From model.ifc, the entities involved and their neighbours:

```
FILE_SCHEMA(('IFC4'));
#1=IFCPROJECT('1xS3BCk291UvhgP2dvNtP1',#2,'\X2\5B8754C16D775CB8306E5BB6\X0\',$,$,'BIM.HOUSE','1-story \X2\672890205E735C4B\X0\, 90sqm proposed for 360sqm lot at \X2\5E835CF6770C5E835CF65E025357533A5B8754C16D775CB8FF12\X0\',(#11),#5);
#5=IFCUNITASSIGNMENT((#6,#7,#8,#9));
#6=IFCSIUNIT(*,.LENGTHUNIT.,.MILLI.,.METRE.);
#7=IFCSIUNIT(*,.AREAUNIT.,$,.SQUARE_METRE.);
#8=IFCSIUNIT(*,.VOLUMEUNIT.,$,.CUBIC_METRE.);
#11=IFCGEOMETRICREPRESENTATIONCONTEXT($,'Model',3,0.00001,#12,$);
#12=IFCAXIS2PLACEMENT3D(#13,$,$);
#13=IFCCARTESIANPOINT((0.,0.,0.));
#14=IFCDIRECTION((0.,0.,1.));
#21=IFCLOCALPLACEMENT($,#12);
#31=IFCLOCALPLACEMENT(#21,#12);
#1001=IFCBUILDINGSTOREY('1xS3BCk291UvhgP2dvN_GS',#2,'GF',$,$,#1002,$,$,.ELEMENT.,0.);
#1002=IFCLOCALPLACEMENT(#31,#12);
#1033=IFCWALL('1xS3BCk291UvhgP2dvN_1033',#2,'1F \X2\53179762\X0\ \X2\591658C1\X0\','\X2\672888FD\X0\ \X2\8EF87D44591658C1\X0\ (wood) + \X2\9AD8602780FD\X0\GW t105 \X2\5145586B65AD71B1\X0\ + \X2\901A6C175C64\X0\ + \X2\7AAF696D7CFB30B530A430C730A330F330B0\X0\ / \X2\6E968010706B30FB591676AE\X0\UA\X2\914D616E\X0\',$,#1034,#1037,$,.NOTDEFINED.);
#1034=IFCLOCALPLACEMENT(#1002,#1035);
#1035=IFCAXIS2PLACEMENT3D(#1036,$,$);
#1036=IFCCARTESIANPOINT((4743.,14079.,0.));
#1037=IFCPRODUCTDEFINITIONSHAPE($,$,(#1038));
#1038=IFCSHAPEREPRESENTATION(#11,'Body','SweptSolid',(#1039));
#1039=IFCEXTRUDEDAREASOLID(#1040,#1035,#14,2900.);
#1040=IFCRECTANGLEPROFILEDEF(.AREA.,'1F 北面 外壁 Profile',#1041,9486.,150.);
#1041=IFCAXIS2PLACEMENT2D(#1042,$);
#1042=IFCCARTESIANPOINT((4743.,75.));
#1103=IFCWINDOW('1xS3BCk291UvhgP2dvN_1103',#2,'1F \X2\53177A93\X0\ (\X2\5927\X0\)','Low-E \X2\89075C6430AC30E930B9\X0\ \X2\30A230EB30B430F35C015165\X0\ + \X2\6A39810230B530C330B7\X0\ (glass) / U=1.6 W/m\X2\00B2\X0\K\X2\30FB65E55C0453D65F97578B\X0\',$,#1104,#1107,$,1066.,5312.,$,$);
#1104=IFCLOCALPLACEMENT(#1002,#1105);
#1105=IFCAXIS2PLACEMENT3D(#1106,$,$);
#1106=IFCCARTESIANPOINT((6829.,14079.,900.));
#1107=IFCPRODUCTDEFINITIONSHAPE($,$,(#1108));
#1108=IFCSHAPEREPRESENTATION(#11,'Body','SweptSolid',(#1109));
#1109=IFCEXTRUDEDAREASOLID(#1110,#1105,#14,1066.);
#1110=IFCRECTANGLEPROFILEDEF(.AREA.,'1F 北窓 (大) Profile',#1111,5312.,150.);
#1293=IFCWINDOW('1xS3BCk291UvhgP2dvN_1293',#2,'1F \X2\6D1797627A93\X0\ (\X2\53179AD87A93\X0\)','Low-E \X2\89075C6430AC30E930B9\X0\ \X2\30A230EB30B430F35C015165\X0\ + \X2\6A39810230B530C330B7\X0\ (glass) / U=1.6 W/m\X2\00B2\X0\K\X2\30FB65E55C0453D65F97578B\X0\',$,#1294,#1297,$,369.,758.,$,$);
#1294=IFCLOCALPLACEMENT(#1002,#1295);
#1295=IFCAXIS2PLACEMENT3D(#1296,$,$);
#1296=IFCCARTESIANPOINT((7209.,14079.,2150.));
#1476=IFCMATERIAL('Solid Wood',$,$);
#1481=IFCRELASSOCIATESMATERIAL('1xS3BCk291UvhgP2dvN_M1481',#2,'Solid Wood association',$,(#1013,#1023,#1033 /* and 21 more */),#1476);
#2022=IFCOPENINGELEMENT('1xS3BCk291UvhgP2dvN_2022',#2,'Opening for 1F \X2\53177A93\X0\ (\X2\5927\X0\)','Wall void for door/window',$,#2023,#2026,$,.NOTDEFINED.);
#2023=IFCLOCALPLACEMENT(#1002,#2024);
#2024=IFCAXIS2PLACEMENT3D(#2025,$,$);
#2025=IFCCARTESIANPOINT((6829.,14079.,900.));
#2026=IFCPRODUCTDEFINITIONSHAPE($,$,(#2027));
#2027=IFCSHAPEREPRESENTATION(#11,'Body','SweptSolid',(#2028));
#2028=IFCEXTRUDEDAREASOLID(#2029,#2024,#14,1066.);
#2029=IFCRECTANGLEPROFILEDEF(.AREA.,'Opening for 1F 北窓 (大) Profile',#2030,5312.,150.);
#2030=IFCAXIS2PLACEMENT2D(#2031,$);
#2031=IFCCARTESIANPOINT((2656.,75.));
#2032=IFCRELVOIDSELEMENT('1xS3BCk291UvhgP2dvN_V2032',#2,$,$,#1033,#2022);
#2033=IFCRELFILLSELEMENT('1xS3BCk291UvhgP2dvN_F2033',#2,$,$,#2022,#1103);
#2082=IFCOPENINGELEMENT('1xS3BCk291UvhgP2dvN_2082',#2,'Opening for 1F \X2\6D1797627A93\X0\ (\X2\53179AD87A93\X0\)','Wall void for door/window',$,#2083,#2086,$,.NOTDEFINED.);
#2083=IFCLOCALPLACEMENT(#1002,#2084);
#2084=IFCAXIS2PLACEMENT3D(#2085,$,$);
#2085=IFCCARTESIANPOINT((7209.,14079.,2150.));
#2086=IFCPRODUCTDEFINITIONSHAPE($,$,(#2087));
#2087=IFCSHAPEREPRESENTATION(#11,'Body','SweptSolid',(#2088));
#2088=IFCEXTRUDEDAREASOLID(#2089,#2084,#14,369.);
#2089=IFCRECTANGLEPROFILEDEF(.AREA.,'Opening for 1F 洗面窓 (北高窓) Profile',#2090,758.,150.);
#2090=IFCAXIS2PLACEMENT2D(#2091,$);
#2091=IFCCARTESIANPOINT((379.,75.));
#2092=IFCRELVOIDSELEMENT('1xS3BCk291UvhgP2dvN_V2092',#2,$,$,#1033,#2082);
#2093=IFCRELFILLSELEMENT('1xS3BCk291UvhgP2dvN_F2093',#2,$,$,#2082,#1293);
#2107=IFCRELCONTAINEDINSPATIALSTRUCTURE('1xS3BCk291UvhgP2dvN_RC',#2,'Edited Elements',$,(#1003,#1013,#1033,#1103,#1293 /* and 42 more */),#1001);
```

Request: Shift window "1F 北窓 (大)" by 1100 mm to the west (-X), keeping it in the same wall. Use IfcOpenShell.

```python
import ifcopenshell
import ifcopenshell.api.geometry
import ifcopenshell.util.placement
import ifcopenshell.util.unit

model = ifcopenshell.open("model.ifc")
unit_scale = ifcopenshell.util.unit.calculate_unit_scale(model)

window = model.by_guid("1xS3BCk291UvhgP2dvN_1103")
opening = window.FillsVoids[0].RelatingOpeningElement
wall = opening.VoidsElements[0].RelatingBuildingElement

wall_matrix = ifcopenshell.util.placement.get_local_placement(wall.ObjectPlacement)
shift = wall_matrix[:3, 0] * -1.1 / unit_scale
before = ifcopenshell.util.placement.get_local_placement(window.ObjectPlacement)[:3, 3].copy()

# The window is not placed relative to its opening, so move both.
for product in (opening, window):
    matrix = ifcopenshell.util.placement.get_local_placement(product.ObjectPlacement)
    matrix[:3, 3] += shift
    ifcopenshell.api.geometry.edit_object_placement(model, product=product, matrix=matrix, is_si=False)

after = ifcopenshell.util.placement.get_local_placement(window.ObjectPlacement)[:3, 3]
print("window moved by", (after - before).round(3) + 0.0)

model.write("model_v2.ifc")
```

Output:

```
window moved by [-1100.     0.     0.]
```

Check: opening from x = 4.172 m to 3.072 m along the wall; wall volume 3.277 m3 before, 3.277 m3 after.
